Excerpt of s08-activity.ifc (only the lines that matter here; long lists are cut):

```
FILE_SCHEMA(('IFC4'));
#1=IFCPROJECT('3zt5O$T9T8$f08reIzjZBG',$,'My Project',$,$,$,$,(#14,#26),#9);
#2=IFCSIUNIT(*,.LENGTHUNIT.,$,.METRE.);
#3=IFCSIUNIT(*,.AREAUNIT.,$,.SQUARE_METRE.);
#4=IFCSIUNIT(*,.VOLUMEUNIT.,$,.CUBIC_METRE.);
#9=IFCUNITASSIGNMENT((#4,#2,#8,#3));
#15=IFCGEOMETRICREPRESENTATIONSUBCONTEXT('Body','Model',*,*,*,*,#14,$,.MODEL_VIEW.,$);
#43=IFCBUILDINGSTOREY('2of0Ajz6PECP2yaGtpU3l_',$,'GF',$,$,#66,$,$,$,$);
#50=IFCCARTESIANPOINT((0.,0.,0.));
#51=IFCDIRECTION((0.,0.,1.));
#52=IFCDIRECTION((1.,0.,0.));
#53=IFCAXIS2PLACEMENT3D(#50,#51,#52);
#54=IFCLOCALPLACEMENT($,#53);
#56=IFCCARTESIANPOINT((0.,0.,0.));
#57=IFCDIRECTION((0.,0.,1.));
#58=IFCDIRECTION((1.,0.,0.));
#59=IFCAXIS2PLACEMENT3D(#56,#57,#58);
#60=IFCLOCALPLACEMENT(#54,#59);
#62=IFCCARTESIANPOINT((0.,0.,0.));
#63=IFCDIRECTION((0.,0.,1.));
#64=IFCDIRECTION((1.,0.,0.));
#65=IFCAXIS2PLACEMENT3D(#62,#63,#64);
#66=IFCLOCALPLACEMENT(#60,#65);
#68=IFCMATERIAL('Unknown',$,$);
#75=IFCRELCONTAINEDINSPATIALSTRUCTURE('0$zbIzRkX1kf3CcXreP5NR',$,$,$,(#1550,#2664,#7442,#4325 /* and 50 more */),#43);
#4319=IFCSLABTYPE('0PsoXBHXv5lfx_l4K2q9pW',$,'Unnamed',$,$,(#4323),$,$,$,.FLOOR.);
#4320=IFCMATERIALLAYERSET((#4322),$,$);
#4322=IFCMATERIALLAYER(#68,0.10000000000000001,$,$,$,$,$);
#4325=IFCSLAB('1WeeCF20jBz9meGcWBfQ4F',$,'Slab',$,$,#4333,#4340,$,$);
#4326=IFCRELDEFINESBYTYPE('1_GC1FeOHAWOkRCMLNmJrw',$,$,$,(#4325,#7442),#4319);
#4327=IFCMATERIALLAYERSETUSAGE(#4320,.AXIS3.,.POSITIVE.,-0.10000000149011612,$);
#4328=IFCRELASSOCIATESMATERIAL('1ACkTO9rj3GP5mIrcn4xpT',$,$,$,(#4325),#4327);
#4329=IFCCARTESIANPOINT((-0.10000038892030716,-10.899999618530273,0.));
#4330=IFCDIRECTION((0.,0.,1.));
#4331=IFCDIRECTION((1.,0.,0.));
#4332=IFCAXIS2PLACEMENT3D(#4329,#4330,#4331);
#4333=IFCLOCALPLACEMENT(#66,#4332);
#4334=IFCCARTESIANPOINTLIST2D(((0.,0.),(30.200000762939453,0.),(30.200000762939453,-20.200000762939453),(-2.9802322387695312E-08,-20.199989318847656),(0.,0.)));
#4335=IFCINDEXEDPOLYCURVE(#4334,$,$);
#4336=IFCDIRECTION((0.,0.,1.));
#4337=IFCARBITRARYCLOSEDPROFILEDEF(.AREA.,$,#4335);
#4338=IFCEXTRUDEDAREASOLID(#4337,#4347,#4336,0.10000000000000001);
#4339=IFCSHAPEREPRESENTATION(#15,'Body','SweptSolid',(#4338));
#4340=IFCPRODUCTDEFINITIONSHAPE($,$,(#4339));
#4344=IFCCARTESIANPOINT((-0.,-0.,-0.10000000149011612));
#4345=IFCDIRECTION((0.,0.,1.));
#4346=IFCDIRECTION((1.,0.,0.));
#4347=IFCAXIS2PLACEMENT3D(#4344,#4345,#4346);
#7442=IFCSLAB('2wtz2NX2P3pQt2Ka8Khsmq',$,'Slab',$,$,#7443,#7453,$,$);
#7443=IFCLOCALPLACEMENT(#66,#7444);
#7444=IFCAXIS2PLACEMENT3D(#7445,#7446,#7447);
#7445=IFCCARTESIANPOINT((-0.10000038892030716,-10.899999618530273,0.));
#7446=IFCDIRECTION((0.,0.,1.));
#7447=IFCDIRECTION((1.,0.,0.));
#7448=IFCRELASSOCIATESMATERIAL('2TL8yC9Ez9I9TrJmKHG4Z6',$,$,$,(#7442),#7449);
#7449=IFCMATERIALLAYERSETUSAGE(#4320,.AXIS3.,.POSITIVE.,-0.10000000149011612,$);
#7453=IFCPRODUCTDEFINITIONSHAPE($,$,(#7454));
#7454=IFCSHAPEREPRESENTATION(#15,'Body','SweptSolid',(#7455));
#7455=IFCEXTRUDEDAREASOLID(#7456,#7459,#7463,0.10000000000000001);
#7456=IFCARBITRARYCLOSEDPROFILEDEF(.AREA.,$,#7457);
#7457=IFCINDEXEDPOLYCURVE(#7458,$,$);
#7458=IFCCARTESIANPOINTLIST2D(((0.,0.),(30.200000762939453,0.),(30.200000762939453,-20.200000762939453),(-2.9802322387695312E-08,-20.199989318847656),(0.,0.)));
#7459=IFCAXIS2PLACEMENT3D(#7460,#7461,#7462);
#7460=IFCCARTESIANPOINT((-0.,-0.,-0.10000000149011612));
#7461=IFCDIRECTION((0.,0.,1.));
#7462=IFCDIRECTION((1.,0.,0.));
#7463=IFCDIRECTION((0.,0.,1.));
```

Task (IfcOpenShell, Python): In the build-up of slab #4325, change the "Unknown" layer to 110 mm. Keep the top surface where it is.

```python
import ifcopenshell
import ifcopenshell.util.element
import ifcopenshell.util.representation
import ifcopenshell.util.unit

model = ifcopenshell.open("s08-activity.ifc")
unit_scale = ifcopenshell.util.unit.calculate_unit_scale(model)

layer_set = model.by_id(4320)
layer = next(l for l in layer_set.MaterialLayers if l.Material and l.Material.Name == "Unknown")
change = 0.11 / unit_scale - layer.LayerThickness
layer.LayerThickness += change

# The layer set is shared, so every slab that uses it gets the new thickness.
slabs = [e for e in ifcopenshell.util.element.get_elements_by_material(model, layer_set) if e.is_a("IfcSlab")]
for slab in sorted(slabs, key=lambda e: e.id()):
    body = ifcopenshell.util.representation.get_representation(slab, "Model", "Body")
    solid = body.Items[0]
    old_depth = solid.Depth
    solid.Depth += change
    # Extruded upwards: lower the start of the extrusion so the top stays.
    x, y, z = solid.Position.Location.Coordinates
    solid.Position.Location = model.createIfcCartesianPoint((x, y, z - change))
    print(slab.id(), f"{old_depth:g} -> {solid.Depth:g}")

# The layers are counted up from the underside, which has moved.
for usage in {ifcopenshell.util.element.get_material(slab) for slab in slabs}:
    usage.OffsetFromReferenceLine -= change

model.write("s08-activity_v2.ifc")
```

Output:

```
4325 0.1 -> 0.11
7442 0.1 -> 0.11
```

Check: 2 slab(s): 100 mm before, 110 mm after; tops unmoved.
